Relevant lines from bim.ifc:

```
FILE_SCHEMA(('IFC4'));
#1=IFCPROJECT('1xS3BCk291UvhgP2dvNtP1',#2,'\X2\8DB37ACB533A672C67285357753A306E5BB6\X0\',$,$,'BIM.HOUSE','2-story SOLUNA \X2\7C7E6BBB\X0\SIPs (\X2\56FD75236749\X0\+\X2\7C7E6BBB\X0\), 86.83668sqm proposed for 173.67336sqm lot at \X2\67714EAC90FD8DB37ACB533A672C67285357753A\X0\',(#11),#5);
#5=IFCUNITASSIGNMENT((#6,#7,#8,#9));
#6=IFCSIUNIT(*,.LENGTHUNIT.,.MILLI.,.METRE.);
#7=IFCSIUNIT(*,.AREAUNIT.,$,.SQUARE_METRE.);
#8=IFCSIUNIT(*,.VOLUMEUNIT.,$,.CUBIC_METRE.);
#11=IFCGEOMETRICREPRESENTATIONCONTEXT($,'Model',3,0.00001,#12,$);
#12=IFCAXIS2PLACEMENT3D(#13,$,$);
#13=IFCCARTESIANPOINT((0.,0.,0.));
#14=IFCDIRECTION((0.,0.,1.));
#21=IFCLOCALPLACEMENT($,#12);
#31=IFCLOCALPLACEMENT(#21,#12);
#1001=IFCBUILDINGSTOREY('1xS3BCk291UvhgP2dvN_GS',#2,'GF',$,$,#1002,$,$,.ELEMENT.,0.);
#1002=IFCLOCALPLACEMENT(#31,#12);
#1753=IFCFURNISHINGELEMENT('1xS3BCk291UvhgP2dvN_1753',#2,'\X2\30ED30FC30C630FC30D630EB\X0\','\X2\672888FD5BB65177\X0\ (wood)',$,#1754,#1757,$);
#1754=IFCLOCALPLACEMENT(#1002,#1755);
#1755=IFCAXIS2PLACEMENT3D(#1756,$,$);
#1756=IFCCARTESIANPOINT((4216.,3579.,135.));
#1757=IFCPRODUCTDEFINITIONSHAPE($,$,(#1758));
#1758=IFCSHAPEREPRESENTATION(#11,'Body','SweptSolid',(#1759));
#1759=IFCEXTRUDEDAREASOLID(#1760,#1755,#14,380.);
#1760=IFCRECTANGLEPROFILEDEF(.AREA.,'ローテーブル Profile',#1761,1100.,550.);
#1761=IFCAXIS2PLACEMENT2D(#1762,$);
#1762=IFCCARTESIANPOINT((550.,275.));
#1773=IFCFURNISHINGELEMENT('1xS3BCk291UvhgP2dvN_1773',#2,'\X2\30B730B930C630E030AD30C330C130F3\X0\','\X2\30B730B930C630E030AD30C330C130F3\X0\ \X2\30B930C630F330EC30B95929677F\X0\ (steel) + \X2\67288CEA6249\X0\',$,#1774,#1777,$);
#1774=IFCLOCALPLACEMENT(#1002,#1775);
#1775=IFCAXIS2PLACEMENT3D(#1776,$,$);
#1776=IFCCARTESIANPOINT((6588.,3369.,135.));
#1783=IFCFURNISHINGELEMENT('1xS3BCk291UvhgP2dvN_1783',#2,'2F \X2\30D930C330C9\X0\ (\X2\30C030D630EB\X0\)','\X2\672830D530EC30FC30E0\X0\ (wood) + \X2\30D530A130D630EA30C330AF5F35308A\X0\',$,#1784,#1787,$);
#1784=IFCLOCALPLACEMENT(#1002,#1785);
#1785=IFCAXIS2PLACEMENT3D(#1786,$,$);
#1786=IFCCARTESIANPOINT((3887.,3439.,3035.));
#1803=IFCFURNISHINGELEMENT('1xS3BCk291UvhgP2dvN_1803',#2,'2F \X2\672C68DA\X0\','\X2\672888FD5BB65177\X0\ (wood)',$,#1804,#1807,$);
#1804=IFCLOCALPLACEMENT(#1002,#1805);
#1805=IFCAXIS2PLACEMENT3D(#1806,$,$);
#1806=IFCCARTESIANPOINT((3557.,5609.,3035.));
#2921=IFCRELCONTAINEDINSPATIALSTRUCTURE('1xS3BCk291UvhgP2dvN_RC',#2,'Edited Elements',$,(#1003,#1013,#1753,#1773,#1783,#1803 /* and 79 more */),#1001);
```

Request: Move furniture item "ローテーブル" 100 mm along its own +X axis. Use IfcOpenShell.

```python
import ifcopenshell
import ifcopenshell.api.geometry
import ifcopenshell.util.placement
import ifcopenshell.util.unit

model = ifcopenshell.open("bim.ifc")
unit_scale = ifcopenshell.util.unit.calculate_unit_scale(model)

item = model.by_guid("1xS3BCk291UvhgP2dvN_1753")
matrix = ifcopenshell.util.placement.get_local_placement(item.ObjectPlacement)
matrix[:3, 3] += matrix[:3, 0] * 0.1 / unit_scale
ifcopenshell.api.geometry.edit_object_placement(model, product=item, matrix=matrix, is_si=False)

print(ifcopenshell.util.placement.get_local_placement(item.ObjectPlacement).round(3) + 0.0)

model.write("bim_rev.ifc")
```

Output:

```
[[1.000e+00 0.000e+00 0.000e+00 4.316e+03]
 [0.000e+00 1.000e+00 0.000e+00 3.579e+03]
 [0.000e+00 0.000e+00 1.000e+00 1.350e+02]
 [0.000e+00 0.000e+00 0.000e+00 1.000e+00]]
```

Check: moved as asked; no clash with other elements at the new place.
